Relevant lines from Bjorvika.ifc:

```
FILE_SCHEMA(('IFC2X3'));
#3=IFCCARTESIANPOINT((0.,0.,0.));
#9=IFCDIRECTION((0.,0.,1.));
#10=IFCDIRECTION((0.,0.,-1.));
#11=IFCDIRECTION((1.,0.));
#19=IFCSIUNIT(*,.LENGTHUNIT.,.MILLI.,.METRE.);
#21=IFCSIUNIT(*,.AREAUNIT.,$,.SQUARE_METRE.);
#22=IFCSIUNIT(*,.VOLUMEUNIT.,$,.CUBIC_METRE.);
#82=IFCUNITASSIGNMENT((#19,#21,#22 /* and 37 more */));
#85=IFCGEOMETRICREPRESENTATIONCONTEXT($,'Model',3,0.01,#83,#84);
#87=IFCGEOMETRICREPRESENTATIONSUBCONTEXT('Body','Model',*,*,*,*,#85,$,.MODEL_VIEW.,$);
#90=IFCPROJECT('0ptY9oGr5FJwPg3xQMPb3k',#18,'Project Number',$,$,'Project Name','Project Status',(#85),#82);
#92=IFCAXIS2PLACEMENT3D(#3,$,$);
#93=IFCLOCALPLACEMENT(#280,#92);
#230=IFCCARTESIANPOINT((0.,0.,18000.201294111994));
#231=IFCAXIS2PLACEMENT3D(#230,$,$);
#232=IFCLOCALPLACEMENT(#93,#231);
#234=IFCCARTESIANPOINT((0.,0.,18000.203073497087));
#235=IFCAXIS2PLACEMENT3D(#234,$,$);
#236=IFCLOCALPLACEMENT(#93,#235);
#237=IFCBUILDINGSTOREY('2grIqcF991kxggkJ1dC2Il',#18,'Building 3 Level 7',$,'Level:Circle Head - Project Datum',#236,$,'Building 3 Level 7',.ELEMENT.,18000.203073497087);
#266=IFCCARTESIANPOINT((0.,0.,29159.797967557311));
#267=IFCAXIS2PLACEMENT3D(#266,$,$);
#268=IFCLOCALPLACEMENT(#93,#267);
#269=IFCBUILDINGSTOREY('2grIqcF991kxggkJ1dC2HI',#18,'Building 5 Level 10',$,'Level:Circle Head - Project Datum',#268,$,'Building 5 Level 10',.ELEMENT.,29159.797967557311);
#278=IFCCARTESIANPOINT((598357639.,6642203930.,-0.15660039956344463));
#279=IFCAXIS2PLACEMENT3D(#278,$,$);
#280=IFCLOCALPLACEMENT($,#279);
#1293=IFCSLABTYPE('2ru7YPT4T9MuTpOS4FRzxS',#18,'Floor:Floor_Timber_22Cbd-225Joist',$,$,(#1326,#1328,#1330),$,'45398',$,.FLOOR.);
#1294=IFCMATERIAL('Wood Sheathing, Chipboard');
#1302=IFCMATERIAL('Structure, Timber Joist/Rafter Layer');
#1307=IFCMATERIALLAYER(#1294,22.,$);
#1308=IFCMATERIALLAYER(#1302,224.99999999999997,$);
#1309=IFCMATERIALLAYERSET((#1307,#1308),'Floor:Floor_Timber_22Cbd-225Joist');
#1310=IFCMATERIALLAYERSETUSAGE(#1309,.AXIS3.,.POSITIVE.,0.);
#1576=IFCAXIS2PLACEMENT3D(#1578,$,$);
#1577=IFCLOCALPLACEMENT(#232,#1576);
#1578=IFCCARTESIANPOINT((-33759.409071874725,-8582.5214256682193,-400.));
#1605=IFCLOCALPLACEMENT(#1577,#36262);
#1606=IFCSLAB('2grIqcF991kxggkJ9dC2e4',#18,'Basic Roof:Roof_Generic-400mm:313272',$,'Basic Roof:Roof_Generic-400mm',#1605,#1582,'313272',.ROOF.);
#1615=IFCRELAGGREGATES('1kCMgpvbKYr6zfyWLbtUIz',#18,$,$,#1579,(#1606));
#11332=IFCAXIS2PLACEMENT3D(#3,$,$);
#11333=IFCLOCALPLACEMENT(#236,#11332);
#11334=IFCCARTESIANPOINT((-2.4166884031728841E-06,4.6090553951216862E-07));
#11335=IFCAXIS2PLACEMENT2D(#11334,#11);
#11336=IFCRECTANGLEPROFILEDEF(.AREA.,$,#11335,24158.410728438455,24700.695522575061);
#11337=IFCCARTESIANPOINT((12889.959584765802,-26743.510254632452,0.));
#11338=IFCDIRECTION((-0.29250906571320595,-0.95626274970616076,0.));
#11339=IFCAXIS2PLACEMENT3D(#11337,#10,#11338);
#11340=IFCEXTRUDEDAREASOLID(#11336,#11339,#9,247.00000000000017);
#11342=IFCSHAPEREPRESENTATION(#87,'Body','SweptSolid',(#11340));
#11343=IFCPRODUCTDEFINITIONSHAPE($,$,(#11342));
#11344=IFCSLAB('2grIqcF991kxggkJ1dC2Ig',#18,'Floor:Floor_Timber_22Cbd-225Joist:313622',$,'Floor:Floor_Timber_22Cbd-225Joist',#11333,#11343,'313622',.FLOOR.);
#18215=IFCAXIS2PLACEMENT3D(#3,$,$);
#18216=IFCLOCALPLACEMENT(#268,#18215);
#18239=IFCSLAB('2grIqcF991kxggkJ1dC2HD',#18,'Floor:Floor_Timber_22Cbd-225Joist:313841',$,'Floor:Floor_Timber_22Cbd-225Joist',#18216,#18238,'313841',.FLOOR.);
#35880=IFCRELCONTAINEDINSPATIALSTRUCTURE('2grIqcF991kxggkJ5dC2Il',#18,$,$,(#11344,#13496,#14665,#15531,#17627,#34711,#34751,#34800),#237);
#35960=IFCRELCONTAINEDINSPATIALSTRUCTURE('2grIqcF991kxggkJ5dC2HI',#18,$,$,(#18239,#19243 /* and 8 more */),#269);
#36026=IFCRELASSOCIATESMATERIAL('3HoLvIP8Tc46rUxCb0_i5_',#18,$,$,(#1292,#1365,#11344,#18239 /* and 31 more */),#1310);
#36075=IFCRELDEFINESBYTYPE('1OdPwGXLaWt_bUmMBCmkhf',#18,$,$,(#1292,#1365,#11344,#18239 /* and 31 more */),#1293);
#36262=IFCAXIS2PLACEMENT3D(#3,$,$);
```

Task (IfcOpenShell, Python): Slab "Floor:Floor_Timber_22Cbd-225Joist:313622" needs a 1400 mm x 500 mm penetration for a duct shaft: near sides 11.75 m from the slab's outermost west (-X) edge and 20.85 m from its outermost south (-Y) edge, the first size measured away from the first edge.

```python
import numpy as np
import ifcopenshell
import ifcopenshell.api.feature
import ifcopenshell.api.geometry
import ifcopenshell.api.root
import ifcopenshell.geom
import ifcopenshell.util.placement
import ifcopenshell.util.representation
import ifcopenshell.util.shape
import ifcopenshell.util.unit

model = ifcopenshell.open("Bjorvika.ifc")
unit_scale = ifcopenshell.util.unit.calculate_unit_scale(model)
settings = ifcopenshell.geom.settings()


def volume(element):
    """Net volume in cubic metres, openings subtracted."""
    shape = ifcopenshell.geom.create_shape(settings, element)
    return ifcopenshell.util.shape.get_volume(shape.geometry)


slab = model.by_guid("2grIqcF991kxggkJ1dC2Ig")
before = volume(slab)

# Extent in the slab's own axes, in metres. The edges named are its -X and -Y sides.
slab_shape = ifcopenshell.geom.create_shape(settings, slab)
vertices = ifcopenshell.util.shape.get_vertices(slab_shape.geometry)
x_min, y_min, bottom = vertices.min(axis=0)
top = vertices[:, 2].max()

opening = ifcopenshell.api.root.create_entity(model, ifc_class="IfcOpeningElement", name="Duct shaft opening")
context = ifcopenshell.util.representation.get_context(model, "Model", "Body", "MODEL_VIEW")
width, depth = 1.4, 0.5
outline = [(0.0, 0.0), (width, 0.0), (width, depth), (0.0, depth), (0.0, 0.0)]
# Overshoot both faces by 50 mm so the cut is clean.
shape = ifcopenshell.api.geometry.add_slab_representation(
    model, context=context, depth=top - bottom + 0.1, polyline=outline
)
ifcopenshell.api.geometry.assign_representation(model, product=opening, representation=shape)

matrix = ifcopenshell.util.placement.get_local_placement(slab.ObjectPlacement)
matrix[:, 3] = matrix @ np.append(np.array([x_min + 11.75, y_min + 20.85, bottom - 0.05]) / unit_scale, 1.0)
ifcopenshell.api.geometry.edit_object_placement(model, product=opening, matrix=matrix, is_si=False)
ifcopenshell.api.feature.add_feature(model, feature=opening, element=slab)

after = volume(slab)

print(f"slab volume {before:.3f} -> {after:.3f} m3")

model.write("Bjorvika_updated.ifc")
```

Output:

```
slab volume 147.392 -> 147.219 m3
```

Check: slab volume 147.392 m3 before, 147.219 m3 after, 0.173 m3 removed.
